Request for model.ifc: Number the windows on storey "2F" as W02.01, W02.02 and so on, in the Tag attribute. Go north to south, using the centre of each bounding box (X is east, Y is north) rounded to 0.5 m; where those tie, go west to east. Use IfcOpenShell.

First a look at what the model holds.

```python
import ifcopenshell
import ifcopenshell.util.element
import ifcopenshell.util.placement

model = ifcopenshell.open("model.ifc")
print(model.schema)
storey = next(s for s in model.by_type("IfcBuildingStorey") if s.Name == "2F")
windows = [e for e in ifcopenshell.util.element.get_decomposition(storey) if e.is_a("IfcWindow")]
for e in sorted(windows, key=lambda e: e.id()):
    origin = ifcopenshell.util.placement.get_local_placement(e.ObjectPlacement)[:3, 3]
    print(e.id(), e.Tag, e.Name, origin.round(2) + 0.0, sep=" | ")
```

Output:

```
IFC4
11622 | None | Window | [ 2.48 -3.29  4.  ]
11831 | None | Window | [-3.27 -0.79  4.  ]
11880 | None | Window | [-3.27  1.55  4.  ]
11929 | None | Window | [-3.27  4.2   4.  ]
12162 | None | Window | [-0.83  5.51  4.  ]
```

```python
import ifcopenshell
import ifcopenshell.geom
import ifcopenshell.util.element
import ifcopenshell.util.shape

model = ifcopenshell.open("model.ifc")
settings = ifcopenshell.geom.settings()
settings.set("use-world-coords", True)


def centre(element):
    shape = ifcopenshell.geom.create_shape(settings, element)
    return ifcopenshell.util.shape.get_bbox_centroid(shape.geometry)


storey = next(s for s in model.by_type("IfcBuildingStorey") if s.Name == "2F")
windows = [e for e in ifcopenshell.util.element.get_decomposition(storey) if e.is_a("IfcWindow")]

# Insertion points can sit at a corner or the storey origin, so sort by the geometry (in metres).
centres = {e: centre(e) for e in windows}
windows.sort(key=lambda e: (-round(centres[e][1] / 0.5), centres[e][0]))

for i, e in enumerate(windows, start=1):
    number = f"W02.{i:02d}"
    e.Tag = number
    print(e.id(), number)

model.write("model-out.ifc")
```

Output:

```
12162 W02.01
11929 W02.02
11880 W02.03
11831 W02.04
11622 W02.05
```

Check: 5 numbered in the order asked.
